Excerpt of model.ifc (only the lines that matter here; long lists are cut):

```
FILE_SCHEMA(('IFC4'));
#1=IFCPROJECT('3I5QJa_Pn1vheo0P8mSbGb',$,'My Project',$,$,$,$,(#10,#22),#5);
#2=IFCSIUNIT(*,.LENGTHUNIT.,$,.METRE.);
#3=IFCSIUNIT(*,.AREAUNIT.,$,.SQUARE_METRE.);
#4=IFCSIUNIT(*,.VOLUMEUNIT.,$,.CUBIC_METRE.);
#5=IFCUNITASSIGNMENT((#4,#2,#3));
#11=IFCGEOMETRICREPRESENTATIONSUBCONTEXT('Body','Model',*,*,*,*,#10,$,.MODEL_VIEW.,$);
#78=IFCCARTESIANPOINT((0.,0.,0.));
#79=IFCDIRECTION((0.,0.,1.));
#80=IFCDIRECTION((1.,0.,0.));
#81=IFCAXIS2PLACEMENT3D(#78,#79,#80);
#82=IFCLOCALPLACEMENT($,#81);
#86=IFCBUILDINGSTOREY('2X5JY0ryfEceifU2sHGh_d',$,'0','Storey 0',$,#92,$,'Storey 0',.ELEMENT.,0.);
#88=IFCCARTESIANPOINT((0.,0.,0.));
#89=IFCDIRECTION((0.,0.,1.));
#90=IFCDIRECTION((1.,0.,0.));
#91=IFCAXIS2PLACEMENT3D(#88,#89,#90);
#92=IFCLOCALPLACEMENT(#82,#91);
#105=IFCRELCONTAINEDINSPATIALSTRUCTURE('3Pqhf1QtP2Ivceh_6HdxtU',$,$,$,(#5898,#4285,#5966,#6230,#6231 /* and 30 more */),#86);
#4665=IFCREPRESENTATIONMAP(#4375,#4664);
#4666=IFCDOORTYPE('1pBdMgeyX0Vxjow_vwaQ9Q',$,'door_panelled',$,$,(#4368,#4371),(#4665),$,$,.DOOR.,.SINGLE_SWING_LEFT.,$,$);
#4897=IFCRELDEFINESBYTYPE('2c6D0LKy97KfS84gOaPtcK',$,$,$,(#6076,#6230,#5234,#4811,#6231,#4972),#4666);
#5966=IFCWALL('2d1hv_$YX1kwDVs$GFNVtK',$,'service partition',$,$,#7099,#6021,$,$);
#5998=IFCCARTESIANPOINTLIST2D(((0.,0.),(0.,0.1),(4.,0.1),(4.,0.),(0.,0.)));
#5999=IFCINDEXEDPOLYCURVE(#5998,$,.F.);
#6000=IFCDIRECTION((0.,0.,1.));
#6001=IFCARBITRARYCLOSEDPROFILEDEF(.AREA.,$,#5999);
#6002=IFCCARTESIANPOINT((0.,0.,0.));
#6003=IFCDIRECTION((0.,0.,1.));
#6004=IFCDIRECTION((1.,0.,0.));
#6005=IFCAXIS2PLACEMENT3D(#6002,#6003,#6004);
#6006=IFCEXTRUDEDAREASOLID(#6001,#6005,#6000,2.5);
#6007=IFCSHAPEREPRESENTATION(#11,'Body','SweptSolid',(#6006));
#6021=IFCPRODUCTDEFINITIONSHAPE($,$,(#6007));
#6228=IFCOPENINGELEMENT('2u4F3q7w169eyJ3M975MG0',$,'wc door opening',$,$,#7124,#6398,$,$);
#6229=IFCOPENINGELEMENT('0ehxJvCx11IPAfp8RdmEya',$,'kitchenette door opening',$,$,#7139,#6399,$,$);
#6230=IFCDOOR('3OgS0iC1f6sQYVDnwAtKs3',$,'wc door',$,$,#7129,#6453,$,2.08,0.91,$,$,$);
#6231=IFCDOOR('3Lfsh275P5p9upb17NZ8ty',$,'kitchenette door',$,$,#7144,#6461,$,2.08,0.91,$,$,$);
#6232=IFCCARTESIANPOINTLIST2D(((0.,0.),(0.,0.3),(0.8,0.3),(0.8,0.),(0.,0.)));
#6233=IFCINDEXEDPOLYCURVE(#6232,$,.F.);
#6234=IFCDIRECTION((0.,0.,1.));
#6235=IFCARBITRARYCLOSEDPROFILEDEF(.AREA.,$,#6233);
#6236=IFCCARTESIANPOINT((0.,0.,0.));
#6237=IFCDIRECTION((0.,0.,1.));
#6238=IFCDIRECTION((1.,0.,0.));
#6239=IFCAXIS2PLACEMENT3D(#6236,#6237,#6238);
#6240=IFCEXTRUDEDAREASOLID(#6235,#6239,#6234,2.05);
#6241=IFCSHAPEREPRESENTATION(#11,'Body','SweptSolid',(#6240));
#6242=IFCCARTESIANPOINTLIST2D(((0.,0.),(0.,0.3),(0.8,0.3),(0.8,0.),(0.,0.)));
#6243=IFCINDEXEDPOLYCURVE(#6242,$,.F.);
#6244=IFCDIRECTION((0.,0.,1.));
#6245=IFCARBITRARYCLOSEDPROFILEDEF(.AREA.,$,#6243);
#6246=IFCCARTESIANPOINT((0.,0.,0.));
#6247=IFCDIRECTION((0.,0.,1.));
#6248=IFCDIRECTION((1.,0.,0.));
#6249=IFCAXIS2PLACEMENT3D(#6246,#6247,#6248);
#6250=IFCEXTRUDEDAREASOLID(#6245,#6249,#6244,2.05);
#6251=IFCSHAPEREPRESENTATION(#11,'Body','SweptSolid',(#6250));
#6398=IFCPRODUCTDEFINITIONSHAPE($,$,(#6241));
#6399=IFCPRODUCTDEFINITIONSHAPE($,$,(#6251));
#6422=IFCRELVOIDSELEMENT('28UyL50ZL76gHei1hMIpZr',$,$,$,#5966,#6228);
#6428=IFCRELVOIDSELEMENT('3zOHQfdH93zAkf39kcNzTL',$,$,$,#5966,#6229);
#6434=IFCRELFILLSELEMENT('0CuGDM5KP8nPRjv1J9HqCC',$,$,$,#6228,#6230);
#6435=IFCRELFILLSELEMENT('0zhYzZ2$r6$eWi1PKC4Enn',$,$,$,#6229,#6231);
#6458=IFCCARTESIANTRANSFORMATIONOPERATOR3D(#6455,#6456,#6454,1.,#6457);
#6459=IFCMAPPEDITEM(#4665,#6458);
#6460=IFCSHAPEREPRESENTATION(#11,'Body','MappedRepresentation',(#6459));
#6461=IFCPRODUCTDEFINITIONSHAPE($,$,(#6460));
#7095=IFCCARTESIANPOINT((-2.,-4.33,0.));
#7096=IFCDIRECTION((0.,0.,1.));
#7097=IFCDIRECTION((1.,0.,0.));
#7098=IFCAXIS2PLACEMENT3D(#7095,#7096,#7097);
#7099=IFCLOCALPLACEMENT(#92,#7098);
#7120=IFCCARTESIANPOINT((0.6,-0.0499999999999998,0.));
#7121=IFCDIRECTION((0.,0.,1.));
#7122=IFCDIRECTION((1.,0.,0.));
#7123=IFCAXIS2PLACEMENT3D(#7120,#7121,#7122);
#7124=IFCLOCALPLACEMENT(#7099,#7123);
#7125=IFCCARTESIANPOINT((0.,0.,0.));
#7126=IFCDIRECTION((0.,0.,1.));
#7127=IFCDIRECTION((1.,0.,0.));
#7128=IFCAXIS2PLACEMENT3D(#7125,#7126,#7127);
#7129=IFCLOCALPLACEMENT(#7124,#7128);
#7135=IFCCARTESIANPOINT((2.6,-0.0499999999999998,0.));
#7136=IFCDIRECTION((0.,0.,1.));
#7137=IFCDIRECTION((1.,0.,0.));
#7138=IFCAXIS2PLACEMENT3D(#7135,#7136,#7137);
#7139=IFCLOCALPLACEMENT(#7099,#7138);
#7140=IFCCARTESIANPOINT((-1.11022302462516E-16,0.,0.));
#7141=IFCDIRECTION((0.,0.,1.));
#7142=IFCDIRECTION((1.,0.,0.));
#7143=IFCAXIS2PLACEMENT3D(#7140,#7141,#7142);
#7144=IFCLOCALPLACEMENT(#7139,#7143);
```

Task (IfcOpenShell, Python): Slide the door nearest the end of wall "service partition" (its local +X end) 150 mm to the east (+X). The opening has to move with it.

```python
import ifcopenshell
import ifcopenshell.api.geometry
import ifcopenshell.util.placement
import ifcopenshell.util.unit

model = ifcopenshell.open("model.ifc")
unit_scale = ifcopenshell.util.unit.calculate_unit_scale(model)

door = model.by_guid("3Lfsh275P5p9upb17NZ8ty")
opening = door.FillsVoids[0].RelatingOpeningElement
wall = opening.VoidsElements[0].RelatingBuildingElement

wall_matrix = ifcopenshell.util.placement.get_local_placement(wall.ObjectPlacement)
shift = wall_matrix[:3, 0] * 0.15 / unit_scale
before = ifcopenshell.util.placement.get_local_placement(door.ObjectPlacement)[:3, 3].copy()

# The door is placed relative to its opening, so it follows when the opening moves.
matrix = ifcopenshell.util.placement.get_local_placement(opening.ObjectPlacement)
matrix[:3, 3] += shift
ifcopenshell.api.geometry.edit_object_placement(
    model, product=opening, matrix=matrix, is_si=False, should_transform_children=True
)

after = ifcopenshell.util.placement.get_local_placement(door.ObjectPlacement)[:3, 3]
print("door moved by", (after - before).round(3) + 0.0)

model.write("model_edited.ifc")
```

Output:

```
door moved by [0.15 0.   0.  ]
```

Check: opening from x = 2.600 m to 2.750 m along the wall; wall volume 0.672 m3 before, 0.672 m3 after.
